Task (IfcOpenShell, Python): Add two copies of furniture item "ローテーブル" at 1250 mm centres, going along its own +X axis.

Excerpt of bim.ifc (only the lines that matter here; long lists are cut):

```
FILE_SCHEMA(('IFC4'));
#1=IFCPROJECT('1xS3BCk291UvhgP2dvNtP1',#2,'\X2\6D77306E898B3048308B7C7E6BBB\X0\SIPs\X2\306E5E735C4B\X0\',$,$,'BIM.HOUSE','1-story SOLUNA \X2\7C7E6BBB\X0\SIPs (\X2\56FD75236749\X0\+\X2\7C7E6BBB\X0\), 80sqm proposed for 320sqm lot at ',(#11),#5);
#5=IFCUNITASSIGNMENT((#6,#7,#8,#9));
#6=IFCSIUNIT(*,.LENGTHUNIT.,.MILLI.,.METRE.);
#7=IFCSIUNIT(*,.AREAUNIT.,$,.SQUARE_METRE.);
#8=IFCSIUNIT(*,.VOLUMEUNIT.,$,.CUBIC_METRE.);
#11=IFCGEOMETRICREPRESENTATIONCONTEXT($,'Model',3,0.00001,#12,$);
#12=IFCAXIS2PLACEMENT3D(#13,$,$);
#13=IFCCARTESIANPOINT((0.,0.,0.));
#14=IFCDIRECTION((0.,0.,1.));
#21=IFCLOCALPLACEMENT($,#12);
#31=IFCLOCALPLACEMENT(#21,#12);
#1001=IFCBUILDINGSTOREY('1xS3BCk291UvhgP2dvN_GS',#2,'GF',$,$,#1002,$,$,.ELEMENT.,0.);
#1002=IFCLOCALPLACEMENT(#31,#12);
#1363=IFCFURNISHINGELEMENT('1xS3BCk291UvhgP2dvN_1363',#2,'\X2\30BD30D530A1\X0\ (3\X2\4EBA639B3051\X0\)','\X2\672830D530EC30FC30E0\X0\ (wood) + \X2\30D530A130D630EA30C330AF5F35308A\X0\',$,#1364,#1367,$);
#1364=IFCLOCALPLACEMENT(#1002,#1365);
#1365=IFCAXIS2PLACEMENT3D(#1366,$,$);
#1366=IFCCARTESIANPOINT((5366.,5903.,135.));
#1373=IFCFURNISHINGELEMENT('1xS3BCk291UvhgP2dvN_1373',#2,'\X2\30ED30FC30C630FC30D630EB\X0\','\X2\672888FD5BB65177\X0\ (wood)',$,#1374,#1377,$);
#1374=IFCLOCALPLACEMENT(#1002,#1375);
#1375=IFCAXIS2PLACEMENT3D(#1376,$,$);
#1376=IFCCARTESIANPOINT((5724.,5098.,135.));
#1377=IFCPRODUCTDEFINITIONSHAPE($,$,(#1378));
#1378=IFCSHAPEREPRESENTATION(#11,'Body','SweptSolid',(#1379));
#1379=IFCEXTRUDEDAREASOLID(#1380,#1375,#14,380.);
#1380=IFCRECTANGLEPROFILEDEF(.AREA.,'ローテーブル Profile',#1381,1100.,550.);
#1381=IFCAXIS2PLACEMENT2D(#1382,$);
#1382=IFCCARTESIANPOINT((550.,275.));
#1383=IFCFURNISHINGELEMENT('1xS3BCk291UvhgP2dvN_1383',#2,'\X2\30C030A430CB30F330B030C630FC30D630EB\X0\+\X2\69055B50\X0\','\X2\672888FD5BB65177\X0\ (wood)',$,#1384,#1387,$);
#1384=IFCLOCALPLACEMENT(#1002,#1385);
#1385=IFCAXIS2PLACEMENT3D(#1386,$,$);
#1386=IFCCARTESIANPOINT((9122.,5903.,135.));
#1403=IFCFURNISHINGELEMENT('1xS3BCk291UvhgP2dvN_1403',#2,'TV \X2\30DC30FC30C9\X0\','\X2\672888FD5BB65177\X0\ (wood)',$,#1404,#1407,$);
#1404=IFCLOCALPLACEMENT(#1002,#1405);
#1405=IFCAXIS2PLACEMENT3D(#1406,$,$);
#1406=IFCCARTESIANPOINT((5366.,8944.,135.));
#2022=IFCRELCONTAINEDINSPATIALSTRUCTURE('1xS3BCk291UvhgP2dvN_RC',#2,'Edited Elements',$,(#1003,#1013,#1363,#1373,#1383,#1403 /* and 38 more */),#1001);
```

```python
import ifcopenshell
import ifcopenshell.api.geometry
import ifcopenshell.api.root
import ifcopenshell.util.element
import ifcopenshell.util.placement
import ifcopenshell.util.unit

model = ifcopenshell.open("bim.ifc")
unit_scale = ifcopenshell.util.unit.calculate_unit_scale(model)


def reuse_history(source, copy):
    """copy_class also copies each property set's owner history, people and application; keep the originals."""
    for rel in copy.IsDefinedBy:
        if rel.is_a("IfcRelDefinesByProperties") and (history := rel.RelatingPropertyDefinition.OwnerHistory):
            rel.RelatingPropertyDefinition.OwnerHistory = source.OwnerHistory
            ifcopenshell.util.element.remove_deep2(model, history)


source = model.by_guid("1xS3BCk291UvhgP2dvN_1373")
base = ifcopenshell.util.placement.get_local_placement(source.ObjectPlacement)
step = base[:3, 0] * 1.25 / unit_scale

for i in range(1, 3):
    copy = ifcopenshell.api.root.copy_class(model, product=source)
    copy.Representation = ifcopenshell.util.element.copy_deep(
        model, source.Representation, exclude=["IfcGeometricRepresentationContext", "IfcRepresentationMap"]
    )
    reuse_history(source, copy)
    matrix = base.copy()
    matrix[:3, 3] += i * step
    print("added at", matrix[:3, 3].round(3) + 0.0)
    ifcopenshell.api.geometry.edit_object_placement(model, product=copy, matrix=matrix, is_si=False)

model.write("bim_rev.ifc")
```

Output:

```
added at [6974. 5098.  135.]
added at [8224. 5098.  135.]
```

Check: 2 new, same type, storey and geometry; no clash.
